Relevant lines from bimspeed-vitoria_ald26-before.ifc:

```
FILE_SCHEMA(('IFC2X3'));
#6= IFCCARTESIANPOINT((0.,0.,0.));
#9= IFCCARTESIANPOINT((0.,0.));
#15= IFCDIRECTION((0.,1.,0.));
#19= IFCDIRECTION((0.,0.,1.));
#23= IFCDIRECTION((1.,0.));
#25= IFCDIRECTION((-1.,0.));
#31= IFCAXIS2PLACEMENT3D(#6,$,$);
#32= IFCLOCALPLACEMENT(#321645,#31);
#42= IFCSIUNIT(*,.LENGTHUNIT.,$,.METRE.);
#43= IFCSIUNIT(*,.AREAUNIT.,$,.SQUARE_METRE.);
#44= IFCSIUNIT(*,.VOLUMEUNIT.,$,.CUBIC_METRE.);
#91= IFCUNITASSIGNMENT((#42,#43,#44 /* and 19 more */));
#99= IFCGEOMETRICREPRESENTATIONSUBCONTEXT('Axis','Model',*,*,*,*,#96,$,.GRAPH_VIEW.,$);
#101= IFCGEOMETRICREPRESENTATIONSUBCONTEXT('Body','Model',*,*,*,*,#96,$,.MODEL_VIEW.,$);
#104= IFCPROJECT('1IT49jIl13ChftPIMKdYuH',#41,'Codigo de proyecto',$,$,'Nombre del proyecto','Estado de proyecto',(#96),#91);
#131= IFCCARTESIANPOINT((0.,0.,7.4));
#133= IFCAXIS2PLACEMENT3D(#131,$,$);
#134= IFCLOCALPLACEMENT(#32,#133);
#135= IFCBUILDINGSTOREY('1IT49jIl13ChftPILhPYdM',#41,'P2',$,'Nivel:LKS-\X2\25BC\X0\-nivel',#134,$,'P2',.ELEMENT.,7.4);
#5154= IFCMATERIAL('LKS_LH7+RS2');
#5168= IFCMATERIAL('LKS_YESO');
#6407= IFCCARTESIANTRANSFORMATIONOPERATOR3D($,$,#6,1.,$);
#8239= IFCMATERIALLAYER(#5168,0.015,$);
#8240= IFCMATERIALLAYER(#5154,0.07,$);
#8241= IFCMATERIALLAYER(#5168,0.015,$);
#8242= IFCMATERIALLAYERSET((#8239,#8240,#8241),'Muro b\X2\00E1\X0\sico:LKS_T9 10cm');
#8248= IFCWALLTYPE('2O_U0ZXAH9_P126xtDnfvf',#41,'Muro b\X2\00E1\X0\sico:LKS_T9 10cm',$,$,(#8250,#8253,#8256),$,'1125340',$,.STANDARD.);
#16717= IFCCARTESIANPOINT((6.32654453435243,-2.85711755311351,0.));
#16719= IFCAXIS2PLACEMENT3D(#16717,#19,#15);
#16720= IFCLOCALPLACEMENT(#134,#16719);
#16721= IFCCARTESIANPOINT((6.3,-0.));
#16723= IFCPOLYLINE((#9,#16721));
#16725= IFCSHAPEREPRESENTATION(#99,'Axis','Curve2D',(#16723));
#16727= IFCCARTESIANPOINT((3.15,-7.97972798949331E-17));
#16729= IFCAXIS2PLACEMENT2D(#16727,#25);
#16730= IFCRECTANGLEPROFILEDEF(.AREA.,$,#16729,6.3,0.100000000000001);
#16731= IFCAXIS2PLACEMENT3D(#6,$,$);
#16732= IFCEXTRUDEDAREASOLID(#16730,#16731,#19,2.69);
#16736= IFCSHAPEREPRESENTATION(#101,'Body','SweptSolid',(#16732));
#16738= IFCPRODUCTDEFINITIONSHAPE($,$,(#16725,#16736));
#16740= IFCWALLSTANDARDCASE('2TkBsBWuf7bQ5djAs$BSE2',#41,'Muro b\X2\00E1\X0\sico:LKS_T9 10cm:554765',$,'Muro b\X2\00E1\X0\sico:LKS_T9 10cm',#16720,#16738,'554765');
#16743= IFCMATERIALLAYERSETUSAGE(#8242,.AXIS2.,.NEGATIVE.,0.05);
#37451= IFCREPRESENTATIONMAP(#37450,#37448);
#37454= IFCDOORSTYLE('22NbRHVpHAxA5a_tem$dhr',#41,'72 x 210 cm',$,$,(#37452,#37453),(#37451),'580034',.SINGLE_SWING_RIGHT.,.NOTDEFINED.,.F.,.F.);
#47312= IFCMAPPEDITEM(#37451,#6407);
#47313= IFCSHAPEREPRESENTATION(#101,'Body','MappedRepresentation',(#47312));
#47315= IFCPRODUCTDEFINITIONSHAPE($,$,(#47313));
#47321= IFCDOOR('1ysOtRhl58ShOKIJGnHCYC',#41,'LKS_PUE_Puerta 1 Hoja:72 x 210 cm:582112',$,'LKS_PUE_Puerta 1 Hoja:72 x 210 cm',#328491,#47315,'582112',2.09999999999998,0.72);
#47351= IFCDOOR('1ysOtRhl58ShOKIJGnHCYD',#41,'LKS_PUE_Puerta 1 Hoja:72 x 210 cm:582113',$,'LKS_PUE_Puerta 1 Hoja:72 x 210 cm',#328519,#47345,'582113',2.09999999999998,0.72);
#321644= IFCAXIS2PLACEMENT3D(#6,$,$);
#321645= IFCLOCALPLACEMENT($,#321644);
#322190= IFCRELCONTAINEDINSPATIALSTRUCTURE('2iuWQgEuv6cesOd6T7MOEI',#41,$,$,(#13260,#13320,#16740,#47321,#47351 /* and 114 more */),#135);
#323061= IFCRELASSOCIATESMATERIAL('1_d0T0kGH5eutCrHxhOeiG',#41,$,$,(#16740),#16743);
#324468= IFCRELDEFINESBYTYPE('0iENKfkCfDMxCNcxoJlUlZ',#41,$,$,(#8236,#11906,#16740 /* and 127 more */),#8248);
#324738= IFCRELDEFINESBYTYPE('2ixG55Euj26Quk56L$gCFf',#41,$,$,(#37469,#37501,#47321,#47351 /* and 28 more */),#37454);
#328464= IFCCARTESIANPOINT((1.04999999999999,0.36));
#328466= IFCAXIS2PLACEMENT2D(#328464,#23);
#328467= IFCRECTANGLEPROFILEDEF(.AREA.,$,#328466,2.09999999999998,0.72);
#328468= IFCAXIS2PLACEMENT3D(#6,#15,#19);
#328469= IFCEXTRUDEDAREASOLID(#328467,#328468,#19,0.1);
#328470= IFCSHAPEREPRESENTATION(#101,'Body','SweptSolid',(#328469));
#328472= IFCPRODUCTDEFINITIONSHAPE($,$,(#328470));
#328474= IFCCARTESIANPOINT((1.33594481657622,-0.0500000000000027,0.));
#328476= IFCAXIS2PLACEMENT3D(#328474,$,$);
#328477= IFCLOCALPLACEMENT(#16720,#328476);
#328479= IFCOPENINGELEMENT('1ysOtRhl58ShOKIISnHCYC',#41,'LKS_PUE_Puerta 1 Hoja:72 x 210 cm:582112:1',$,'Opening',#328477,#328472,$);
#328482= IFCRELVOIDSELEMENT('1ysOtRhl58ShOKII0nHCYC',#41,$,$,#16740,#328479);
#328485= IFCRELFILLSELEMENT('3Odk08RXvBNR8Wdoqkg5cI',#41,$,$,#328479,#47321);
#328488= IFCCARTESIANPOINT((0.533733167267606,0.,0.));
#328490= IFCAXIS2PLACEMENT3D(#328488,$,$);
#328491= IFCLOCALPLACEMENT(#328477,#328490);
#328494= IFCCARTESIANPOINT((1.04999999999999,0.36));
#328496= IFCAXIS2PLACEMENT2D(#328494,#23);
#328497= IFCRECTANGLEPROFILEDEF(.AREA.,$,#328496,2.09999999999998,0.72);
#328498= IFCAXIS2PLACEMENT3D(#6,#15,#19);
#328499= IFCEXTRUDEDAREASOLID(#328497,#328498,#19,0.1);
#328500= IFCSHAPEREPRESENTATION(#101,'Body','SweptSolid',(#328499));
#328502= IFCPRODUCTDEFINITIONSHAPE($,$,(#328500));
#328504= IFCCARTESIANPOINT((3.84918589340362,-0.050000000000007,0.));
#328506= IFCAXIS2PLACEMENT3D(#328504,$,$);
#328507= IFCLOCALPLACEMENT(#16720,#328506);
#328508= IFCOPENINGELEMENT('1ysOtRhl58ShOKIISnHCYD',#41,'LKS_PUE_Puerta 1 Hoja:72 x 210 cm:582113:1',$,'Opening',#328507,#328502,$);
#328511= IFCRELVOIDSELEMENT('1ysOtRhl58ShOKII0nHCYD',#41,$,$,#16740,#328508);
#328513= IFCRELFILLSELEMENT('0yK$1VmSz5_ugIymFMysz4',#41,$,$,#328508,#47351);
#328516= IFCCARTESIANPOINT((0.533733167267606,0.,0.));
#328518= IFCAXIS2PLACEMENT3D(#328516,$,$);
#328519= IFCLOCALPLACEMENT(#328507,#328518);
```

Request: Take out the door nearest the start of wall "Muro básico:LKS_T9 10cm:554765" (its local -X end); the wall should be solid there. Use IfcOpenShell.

```python
import ifcopenshell
import ifcopenshell.api.feature
import ifcopenshell.api.root
import ifcopenshell.geom
import ifcopenshell.util.shape

model = ifcopenshell.open("bimspeed-vitoria_ald26-before.ifc")
settings = ifcopenshell.geom.settings()


def volume(element):
    """Net volume in cubic metres, openings subtracted."""
    shape = ifcopenshell.geom.create_shape(settings, element)
    return ifcopenshell.util.shape.get_volume(shape.geometry)


door = model.by_guid("1ysOtRhl58ShOKIJGnHCYC")
opening = door.FillsVoids[0].RelatingOpeningElement
wall = opening.VoidsElements[0].RelatingBuildingElement
before = volume(wall)

ifcopenshell.api.root.remove_product(model, product=door)
ifcopenshell.api.feature.remove_feature(model, feature=opening)

after = volume(wall)

print(f"wall volume {before:.3f} -> {after:.3f} m3")

model.write("bimspeed-vitoria_ald26-before_v2.ifc")
```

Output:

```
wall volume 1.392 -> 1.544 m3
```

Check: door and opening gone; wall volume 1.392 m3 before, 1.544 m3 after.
